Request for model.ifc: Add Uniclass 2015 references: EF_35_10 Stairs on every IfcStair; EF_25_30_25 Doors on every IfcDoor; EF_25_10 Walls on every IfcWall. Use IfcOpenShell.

First a look at what the model holds.

```python
import ifcopenshell

model = ifcopenshell.open("model.ifc")
print(model.schema)
print("classifications:", [c.Name for c in model.by_type("IfcClassification")])
for ifc_class in ("IfcDoor", "IfcRoof", "IfcStair", "IfcWall", "IfcWindow"):
    print(ifc_class, len(model.by_type(ifc_class)))
```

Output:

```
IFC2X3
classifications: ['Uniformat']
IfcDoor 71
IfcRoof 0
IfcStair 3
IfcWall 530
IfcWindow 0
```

```python
import ifcopenshell
import ifcopenshell.api.classification

model = ifcopenshell.open("model.ifc")

# IFC2X3 requires Source and Edition and has no link from the project to the system.
system = model.create_entity("IfcClassification", Source="NBS", Edition="2015", Name="Uniclass 2015")

codes = {
    "IfcStair": ("EF_35_10", "Stairs"),
    "IfcDoor": ("EF_25_30_25", "Doors"),
    "IfcWall": ("EF_25_10", "Walls"),
}
for ifc_class, (code, name) in codes.items():
    products = model.by_type(ifc_class)
    ifcopenshell.api.classification.add_reference(
        model, products=products, classification=system, identification=code, name=name
    )
    print(code, len(products))

model.write("model_v2.ifc")
```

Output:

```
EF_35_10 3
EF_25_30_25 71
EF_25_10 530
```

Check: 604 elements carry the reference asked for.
